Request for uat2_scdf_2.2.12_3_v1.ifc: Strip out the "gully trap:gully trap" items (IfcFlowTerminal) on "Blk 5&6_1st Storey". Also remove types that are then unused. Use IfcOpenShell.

First a look at what the model holds.

```python
import ifcopenshell
import ifcopenshell.util.element

model = ifcopenshell.open("uat2_scdf_2.2.12_3_v1.ifc")
print(model.schema)
storey = next(s for s in model.by_type("IfcBuildingStorey") if s.Name == "Blk 5&6_1st Storey")
terminals = [e for e in ifcopenshell.util.element.get_decomposition(storey) if e.is_a("IfcFlowTerminal")]
seen = {}
for e in terminals:
    element_type = ifcopenshell.util.element.get_type(e)
    name = element_type.Name if element_type not in (None, e) else None
    seen[name] = seen.get(name, 0) + 1
for name, count in sorted(seen.items(), key=str):
    print(count, "x", name)
```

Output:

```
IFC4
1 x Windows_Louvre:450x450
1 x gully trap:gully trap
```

```python
import ifcopenshell
import ifcopenshell.api.root
import ifcopenshell.util.element

model = ifcopenshell.open("uat2_scdf_2.2.12_3_v1.ifc")

storey = next(s for s in model.by_type("IfcBuildingStorey") if s.Name == "Blk 5&6_1st Storey")
terminals = [e for e in ifcopenshell.util.element.get_decomposition(storey) if e.is_a("IfcFlowTerminal")]
targets = [e for e in terminals if (t := ifcopenshell.util.element.get_type(e)) not in (None, e) and t.Name == "gully trap:gully trap"]
types = {ifcopenshell.util.element.get_type(e) for e in targets} - {None, *targets}

for e in targets:
    ifcopenshell.api.root.remove_product(model, product=e)
print(len(targets), "removed")

unused = [t for t in types if not ifcopenshell.util.element.get_types(t)]
for t in unused:
    ifcopenshell.api.root.remove_product(model, product=t)
print(len(unused), "unused types removed")

model.write("uat2_scdf_2.2.12_3_v1_rev.ifc")
```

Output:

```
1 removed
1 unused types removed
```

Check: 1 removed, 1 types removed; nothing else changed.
